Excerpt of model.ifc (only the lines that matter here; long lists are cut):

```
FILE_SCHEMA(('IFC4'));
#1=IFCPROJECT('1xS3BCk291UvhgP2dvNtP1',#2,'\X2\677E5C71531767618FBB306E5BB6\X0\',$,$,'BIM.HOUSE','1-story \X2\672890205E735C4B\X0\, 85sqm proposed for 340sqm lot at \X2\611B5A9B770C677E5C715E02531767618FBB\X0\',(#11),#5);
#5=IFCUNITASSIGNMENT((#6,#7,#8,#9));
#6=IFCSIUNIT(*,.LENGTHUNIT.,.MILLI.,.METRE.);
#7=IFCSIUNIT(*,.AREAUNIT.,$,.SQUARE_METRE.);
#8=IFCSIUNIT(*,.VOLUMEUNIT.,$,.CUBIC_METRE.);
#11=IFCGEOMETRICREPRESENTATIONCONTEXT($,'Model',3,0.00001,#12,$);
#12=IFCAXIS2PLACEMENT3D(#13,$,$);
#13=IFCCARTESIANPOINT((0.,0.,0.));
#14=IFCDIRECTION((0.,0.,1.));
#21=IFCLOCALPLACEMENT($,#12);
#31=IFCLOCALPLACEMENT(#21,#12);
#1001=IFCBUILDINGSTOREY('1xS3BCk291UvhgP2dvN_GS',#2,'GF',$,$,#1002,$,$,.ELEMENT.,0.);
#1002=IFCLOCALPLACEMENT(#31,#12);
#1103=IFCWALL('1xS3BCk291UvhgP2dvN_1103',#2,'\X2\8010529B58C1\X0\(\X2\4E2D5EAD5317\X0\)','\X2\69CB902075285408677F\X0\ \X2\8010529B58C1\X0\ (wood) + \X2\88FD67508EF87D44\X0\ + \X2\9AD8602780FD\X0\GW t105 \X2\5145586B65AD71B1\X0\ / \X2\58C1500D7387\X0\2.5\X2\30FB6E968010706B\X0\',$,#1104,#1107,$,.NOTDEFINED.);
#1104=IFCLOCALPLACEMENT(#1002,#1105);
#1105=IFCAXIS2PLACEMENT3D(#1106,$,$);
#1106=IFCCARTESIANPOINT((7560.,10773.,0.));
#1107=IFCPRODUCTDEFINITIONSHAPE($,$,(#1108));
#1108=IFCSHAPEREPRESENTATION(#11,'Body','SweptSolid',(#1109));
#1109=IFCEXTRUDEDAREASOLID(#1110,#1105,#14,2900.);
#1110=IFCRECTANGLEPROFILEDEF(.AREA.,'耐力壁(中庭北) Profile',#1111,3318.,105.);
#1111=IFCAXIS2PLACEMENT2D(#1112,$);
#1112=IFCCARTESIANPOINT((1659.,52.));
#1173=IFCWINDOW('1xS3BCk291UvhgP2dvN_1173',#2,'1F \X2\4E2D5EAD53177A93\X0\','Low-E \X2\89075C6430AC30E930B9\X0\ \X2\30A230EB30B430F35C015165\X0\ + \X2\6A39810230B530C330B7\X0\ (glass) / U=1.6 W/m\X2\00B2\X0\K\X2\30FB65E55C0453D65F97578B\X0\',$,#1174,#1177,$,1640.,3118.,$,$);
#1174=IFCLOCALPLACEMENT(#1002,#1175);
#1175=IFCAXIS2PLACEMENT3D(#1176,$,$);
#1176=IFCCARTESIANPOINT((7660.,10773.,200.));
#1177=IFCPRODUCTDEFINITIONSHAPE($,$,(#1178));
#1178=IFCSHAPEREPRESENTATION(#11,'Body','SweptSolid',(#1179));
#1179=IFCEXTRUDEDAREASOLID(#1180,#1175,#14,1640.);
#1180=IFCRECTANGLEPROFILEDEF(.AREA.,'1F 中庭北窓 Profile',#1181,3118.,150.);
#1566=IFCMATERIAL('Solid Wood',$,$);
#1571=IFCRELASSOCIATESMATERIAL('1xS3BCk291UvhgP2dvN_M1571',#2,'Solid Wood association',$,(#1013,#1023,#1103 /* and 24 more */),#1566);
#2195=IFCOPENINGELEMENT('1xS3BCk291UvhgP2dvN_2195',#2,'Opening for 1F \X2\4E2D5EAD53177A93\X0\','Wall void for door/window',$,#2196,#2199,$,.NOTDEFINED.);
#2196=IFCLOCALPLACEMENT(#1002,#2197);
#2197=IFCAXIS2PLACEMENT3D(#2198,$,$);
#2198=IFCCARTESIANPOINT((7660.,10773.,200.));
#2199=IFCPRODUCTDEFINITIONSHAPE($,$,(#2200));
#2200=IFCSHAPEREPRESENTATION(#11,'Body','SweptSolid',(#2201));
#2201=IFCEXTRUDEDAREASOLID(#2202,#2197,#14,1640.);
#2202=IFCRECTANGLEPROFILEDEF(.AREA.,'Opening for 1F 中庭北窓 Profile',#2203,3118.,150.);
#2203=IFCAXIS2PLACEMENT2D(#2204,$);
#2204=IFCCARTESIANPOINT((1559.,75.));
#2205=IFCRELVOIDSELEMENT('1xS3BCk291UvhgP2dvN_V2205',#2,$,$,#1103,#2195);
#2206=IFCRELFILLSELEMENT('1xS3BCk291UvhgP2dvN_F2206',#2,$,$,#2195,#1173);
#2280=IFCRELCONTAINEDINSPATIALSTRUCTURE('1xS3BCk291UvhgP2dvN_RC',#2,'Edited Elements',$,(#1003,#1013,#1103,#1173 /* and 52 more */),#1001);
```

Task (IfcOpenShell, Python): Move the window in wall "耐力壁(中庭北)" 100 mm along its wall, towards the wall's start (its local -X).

```python
import ifcopenshell
import ifcopenshell.api.geometry
import ifcopenshell.util.placement
import ifcopenshell.util.unit

model = ifcopenshell.open("model.ifc")
unit_scale = ifcopenshell.util.unit.calculate_unit_scale(model)

window = model.by_id(1173)
opening = window.FillsVoids[0].RelatingOpeningElement
wall = opening.VoidsElements[0].RelatingBuildingElement

wall_matrix = ifcopenshell.util.placement.get_local_placement(wall.ObjectPlacement)
shift = wall_matrix[:3, 0] * -0.1 / unit_scale
before = ifcopenshell.util.placement.get_local_placement(window.ObjectPlacement)[:3, 3].copy()

# The window is not placed relative to its opening, so move both.
for product in (opening, window):
    matrix = ifcopenshell.util.placement.get_local_placement(product.ObjectPlacement)
    matrix[:3, 3] += shift
    ifcopenshell.api.geometry.edit_object_placement(model, product=product, matrix=matrix, is_si=False)

after = ifcopenshell.util.placement.get_local_placement(window.ObjectPlacement)[:3, 3]
print("window moved by", (after - before).round(3) + 0.0)

model.write("model_updated.ifc")
```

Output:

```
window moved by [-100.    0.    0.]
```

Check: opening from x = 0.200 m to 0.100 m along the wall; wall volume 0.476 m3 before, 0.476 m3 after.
